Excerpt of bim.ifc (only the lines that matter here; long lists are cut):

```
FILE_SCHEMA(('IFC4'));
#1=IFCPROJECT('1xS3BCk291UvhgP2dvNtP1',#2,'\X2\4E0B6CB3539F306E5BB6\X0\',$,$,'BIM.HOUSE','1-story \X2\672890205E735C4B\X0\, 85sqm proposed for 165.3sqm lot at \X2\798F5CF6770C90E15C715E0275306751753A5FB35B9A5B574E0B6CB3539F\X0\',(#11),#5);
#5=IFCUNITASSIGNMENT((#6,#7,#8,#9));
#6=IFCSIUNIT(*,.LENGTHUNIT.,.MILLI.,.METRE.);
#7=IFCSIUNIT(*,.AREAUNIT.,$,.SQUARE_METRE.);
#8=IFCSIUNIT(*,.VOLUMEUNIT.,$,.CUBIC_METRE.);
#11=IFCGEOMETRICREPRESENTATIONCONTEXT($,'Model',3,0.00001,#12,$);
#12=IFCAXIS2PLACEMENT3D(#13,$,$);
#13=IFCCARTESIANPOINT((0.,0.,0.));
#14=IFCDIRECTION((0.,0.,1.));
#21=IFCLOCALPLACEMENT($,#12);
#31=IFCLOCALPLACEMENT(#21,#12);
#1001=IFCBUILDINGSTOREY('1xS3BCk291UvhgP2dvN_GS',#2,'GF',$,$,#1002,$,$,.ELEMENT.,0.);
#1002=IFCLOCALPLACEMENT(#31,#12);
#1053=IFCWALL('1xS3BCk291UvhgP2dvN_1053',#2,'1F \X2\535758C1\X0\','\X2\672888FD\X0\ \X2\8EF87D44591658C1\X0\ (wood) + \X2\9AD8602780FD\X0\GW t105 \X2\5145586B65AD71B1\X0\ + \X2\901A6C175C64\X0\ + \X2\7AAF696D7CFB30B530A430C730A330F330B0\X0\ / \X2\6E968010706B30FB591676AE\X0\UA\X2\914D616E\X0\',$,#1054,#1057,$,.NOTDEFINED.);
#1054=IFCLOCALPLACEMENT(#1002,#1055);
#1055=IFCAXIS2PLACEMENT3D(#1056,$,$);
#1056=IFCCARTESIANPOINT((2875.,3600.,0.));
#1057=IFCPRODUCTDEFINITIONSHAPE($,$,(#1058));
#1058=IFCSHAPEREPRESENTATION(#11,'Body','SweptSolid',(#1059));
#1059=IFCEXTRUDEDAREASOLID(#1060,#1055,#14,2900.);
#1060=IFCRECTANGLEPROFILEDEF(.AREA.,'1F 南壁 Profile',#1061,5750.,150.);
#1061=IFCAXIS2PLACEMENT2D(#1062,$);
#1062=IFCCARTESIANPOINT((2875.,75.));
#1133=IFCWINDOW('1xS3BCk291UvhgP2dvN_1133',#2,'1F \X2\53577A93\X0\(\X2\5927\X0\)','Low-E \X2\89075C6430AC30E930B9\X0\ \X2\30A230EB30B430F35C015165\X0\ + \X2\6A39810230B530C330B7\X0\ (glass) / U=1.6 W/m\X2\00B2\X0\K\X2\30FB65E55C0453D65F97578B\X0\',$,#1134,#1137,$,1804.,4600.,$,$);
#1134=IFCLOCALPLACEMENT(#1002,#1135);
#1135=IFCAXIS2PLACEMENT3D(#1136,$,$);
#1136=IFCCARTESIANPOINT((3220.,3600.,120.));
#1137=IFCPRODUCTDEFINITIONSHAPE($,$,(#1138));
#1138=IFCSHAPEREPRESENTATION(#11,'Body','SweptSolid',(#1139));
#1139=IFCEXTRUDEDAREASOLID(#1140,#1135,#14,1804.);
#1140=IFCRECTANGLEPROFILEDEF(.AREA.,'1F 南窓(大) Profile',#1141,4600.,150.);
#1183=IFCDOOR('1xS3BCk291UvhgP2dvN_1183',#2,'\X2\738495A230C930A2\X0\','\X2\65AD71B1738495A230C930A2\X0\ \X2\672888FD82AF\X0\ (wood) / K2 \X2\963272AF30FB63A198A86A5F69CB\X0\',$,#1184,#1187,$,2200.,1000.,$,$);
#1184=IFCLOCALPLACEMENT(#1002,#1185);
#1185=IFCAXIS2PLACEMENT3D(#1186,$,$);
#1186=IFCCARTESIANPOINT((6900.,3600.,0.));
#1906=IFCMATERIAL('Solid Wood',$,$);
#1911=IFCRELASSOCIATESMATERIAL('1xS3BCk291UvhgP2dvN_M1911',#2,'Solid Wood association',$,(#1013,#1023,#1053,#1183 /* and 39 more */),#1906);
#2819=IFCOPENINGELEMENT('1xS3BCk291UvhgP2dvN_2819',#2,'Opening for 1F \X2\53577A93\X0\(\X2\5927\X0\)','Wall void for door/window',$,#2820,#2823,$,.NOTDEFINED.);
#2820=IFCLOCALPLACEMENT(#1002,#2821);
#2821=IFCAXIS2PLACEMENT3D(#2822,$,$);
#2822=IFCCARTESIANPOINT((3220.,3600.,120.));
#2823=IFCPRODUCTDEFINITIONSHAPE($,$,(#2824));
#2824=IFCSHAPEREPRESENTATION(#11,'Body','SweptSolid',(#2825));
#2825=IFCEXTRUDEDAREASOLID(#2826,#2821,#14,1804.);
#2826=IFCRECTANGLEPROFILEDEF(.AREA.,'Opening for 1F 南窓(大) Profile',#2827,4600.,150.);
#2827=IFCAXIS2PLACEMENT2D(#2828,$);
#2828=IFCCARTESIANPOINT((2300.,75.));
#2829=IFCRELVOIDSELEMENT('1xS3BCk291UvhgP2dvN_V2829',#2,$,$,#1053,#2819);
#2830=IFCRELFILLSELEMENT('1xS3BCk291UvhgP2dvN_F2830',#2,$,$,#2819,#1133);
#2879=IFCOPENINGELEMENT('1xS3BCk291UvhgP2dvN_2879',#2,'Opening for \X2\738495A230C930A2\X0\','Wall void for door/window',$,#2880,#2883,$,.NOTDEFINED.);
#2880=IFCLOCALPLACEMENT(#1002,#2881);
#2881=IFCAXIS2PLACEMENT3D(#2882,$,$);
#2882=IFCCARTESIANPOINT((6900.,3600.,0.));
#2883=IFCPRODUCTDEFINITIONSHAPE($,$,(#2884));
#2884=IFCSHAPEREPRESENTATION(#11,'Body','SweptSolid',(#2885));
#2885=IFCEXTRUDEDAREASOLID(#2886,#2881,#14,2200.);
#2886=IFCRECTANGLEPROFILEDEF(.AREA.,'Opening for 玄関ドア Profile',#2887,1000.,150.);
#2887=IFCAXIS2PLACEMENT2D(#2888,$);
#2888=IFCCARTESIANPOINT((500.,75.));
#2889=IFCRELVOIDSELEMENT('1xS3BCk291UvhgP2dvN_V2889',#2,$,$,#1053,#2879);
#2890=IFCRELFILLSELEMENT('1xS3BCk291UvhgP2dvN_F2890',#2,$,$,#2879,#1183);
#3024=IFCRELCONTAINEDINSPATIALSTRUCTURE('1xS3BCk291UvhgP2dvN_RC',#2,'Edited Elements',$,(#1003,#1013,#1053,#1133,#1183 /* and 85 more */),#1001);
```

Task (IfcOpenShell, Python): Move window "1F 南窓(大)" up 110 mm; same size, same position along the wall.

```python
import numpy as np
import ifcopenshell
import ifcopenshell.api.geometry
import ifcopenshell.util.placement
import ifcopenshell.util.unit

model = ifcopenshell.open("bim.ifc")
unit_scale = ifcopenshell.util.unit.calculate_unit_scale(model)

window = model.by_guid("1xS3BCk291UvhgP2dvN_1133")
opening = window.FillsVoids[0].RelatingOpeningElement
dz = 0.11 / unit_scale

shift = np.array([0.0, 0.0, dz])
# The window is not placed relative to its opening, so move both.
for product in (opening, window):
    matrix = ifcopenshell.util.placement.get_local_placement(product.ObjectPlacement)
    matrix[:3, 3] += shift
    ifcopenshell.api.geometry.edit_object_placement(model, product=product, matrix=matrix, is_si=False)

print(f"moved by {dz * unit_scale:+.3f} m")

model.write("bim_edited.ifc")
```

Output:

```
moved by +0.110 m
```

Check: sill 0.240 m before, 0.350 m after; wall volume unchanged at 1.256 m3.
